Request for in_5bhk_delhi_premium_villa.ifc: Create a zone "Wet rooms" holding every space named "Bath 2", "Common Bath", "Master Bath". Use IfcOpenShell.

First a look at what the model holds.

```python
import ifcopenshell

model = ifcopenshell.open("in_5bhk_delhi_premium_villa.ifc")
print(model.schema)
seen = {}
for space in model.by_type("IfcSpace"):
    seen[space.LongName] = seen.get(space.LongName, 0) + 1
for name, count in sorted(seen.items(), key=str):
    print(count, "x", name)
print("zones:", [z.Name for z in model.by_type("IfcZone")][:20])
```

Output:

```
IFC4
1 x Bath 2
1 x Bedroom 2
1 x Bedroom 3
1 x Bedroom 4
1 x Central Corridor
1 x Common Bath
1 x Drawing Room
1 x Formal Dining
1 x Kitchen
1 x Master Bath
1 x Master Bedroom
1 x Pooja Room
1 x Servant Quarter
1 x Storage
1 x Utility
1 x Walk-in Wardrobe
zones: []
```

```python
import ifcopenshell
import ifcopenshell.api.group
import ifcopenshell.api.root

model = ifcopenshell.open("in_5bhk_delhi_premium_villa.ifc")

names = {"Bath 2", "Common Bath", "Master Bath"}
spaces = [s for s in model.by_type("IfcSpace") if s.LongName in names]

zone = ifcopenshell.api.root.create_entity(model, ifc_class="IfcZone", name="Wet rooms")
ifcopenshell.api.group.assign_group(model, products=spaces, group=zone)
print(len(spaces), "spaces in", zone.Name)

model.write("in_5bhk_delhi_premium_villa_updated.ifc")
```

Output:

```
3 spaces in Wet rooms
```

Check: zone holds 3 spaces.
